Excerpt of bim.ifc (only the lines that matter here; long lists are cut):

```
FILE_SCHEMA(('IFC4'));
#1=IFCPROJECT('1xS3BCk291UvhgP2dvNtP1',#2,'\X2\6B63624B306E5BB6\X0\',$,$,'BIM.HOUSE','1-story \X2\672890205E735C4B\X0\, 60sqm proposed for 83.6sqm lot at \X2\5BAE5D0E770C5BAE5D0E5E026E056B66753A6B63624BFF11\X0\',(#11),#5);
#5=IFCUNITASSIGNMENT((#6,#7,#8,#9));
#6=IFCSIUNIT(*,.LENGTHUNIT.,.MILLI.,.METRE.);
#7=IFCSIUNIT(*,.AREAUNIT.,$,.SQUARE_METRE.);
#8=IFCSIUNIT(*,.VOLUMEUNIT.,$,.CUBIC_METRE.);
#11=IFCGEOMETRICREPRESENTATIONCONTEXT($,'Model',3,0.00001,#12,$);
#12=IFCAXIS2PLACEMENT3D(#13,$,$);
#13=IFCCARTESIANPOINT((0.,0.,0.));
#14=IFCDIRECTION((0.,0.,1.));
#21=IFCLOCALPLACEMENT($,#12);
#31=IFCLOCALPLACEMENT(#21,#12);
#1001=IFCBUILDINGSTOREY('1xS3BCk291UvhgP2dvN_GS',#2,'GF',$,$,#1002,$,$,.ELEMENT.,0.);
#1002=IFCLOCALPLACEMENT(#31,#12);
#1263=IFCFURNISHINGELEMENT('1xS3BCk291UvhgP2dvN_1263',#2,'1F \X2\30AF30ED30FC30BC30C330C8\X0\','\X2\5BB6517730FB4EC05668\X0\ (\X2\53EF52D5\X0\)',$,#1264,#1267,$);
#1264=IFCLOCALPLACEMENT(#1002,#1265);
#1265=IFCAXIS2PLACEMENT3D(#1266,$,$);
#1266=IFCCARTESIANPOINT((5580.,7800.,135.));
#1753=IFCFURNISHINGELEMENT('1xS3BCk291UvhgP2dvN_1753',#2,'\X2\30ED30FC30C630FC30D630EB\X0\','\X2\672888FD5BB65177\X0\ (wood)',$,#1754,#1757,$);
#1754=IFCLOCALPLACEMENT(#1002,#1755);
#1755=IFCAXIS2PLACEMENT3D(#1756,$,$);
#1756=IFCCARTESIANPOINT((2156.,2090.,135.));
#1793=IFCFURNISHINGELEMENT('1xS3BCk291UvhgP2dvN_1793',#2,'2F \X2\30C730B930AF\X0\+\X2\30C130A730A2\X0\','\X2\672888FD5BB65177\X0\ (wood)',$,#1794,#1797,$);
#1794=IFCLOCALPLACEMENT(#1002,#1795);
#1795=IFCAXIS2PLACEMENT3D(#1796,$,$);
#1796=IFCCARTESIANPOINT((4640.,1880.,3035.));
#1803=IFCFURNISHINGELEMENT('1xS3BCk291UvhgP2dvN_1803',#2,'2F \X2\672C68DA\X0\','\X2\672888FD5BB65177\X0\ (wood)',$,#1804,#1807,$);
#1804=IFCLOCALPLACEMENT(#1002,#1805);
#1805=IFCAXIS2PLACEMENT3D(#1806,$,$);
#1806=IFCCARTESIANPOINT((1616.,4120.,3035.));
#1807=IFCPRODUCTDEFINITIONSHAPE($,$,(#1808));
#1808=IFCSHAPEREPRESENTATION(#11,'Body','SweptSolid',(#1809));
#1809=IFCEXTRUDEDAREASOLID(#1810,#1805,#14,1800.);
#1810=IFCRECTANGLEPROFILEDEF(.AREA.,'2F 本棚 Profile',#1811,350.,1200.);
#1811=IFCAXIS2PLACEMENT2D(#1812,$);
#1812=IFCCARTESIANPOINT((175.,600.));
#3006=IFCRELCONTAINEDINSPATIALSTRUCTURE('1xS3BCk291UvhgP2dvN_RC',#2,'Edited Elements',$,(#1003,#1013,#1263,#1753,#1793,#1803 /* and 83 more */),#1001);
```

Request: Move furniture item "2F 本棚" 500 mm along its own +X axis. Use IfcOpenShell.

```python
import ifcopenshell
import ifcopenshell.api.geometry
import ifcopenshell.util.placement
import ifcopenshell.util.unit

model = ifcopenshell.open("bim.ifc")
unit_scale = ifcopenshell.util.unit.calculate_unit_scale(model)

item = model.by_guid("1xS3BCk291UvhgP2dvN_1803")
matrix = ifcopenshell.util.placement.get_local_placement(item.ObjectPlacement)
matrix[:3, 3] += matrix[:3, 0] * 0.5 / unit_scale
ifcopenshell.api.geometry.edit_object_placement(model, product=item, matrix=matrix, is_si=False)

print(ifcopenshell.util.placement.get_local_placement(item.ObjectPlacement).round(3) + 0.0)

model.write("bim_edited.ifc")
```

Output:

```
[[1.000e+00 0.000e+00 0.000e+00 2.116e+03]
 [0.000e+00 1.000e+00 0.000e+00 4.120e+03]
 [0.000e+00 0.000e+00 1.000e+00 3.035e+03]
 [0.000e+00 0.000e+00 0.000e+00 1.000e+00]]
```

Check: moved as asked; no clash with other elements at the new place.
